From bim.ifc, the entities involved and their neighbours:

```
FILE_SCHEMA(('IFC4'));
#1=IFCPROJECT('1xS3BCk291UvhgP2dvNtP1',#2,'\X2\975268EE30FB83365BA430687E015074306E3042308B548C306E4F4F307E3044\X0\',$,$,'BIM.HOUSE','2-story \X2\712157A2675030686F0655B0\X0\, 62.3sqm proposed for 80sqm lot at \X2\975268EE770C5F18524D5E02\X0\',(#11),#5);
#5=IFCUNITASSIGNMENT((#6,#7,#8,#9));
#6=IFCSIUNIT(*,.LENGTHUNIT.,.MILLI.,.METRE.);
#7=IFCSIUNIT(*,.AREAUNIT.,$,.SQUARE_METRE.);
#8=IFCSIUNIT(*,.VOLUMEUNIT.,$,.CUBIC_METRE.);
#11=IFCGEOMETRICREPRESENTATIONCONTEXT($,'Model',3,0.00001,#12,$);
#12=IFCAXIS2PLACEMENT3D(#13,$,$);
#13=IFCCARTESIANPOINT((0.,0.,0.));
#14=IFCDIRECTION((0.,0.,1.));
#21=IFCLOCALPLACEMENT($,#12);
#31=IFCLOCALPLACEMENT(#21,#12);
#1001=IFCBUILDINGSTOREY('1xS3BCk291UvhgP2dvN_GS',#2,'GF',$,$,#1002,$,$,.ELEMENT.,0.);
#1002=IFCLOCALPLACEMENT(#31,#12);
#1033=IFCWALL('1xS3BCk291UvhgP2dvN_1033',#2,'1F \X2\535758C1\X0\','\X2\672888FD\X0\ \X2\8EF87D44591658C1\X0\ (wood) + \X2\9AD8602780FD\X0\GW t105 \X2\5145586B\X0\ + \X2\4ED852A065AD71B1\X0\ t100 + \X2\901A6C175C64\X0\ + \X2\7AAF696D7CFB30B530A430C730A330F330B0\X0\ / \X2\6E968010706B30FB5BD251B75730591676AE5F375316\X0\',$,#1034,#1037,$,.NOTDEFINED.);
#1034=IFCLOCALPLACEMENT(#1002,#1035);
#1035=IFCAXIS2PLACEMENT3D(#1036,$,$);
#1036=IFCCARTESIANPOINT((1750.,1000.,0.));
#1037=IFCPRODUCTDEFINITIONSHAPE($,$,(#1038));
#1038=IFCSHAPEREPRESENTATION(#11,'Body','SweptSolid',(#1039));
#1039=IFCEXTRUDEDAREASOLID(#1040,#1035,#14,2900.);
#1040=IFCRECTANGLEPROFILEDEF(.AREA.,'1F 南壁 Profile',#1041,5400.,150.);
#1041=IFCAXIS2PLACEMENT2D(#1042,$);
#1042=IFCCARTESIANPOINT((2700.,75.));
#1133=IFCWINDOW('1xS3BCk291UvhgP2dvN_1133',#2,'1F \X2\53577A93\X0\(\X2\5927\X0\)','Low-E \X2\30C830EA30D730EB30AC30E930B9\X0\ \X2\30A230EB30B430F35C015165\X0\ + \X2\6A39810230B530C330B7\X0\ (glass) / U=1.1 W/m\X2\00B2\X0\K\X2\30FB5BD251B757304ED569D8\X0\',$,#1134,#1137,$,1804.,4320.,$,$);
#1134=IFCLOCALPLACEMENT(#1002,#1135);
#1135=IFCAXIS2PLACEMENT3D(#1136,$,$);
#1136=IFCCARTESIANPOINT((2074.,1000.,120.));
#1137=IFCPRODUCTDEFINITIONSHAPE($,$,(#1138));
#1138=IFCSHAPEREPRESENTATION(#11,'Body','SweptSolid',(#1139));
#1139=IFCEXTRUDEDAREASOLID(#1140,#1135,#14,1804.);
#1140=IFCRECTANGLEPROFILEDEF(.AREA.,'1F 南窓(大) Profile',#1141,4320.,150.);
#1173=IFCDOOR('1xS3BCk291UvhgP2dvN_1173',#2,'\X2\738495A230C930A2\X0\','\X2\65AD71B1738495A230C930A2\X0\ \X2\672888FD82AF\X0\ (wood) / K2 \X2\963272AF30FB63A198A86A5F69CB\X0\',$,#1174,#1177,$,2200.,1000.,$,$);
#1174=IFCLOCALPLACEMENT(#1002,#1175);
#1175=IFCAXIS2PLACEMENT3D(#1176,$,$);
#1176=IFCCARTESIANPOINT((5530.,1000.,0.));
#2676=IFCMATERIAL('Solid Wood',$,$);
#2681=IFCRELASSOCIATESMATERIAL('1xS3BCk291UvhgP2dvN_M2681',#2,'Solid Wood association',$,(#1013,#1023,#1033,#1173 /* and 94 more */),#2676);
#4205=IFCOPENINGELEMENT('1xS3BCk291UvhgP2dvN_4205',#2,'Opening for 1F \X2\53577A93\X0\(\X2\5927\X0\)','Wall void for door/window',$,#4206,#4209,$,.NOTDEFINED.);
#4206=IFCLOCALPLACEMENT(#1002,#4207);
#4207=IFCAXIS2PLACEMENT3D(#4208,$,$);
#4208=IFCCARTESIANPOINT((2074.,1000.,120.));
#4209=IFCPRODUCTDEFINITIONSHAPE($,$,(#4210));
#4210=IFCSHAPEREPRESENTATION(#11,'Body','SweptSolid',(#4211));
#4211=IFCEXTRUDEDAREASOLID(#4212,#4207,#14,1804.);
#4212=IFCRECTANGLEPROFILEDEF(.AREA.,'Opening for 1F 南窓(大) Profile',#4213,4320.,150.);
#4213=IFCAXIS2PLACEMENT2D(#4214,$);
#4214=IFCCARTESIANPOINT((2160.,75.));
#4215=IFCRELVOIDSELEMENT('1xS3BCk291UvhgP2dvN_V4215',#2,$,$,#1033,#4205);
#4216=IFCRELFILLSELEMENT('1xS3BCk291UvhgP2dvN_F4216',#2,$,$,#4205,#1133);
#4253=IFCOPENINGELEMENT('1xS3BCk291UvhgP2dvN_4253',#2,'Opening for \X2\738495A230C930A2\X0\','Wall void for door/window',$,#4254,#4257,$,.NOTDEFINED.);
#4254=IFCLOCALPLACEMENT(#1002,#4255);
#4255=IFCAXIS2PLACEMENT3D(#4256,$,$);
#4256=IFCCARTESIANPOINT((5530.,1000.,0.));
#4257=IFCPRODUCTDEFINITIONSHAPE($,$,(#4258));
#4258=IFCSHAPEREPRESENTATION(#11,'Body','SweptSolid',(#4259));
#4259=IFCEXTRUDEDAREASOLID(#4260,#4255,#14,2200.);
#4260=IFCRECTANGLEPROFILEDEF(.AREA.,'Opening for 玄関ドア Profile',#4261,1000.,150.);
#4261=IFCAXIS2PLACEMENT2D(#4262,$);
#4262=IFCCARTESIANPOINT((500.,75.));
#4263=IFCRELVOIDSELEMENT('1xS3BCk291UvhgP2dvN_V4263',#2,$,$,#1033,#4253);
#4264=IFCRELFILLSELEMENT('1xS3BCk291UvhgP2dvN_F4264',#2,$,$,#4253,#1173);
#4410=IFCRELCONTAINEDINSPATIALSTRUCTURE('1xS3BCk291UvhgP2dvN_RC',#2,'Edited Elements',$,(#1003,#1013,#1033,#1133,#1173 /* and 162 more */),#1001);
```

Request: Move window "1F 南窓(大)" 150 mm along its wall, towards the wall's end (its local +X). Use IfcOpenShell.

```python
import ifcopenshell
import ifcopenshell.api.geometry
import ifcopenshell.util.placement
import ifcopenshell.util.unit

model = ifcopenshell.open("bim.ifc")
unit_scale = ifcopenshell.util.unit.calculate_unit_scale(model)

window = model.by_guid("1xS3BCk291UvhgP2dvN_1133")
opening = window.FillsVoids[0].RelatingOpeningElement
wall = opening.VoidsElements[0].RelatingBuildingElement

wall_matrix = ifcopenshell.util.placement.get_local_placement(wall.ObjectPlacement)
shift = wall_matrix[:3, 0] * 0.15 / unit_scale
before = ifcopenshell.util.placement.get_local_placement(window.ObjectPlacement)[:3, 3].copy()

# The window is not placed relative to its opening, so move both.
for product in (opening, window):
    matrix = ifcopenshell.util.placement.get_local_placement(product.ObjectPlacement)
    matrix[:3, 3] += shift
    ifcopenshell.api.geometry.edit_object_placement(model, product=product, matrix=matrix, is_si=False)

after = ifcopenshell.util.placement.get_local_placement(window.ObjectPlacement)[:3, 3]
print("window moved by", (after - before).round(3) + 0.0)

model.write("bim_edited.ifc")
```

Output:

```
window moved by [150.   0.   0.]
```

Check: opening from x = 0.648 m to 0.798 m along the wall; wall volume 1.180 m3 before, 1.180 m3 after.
